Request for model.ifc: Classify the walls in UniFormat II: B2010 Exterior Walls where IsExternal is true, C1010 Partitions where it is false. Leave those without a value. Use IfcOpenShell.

First a look at what the model holds.

```python
import ifcopenshell
import ifcopenshell.util.element

model = ifcopenshell.open("model.ifc")
print(model.schema)
print("classifications:", [c.Name for c in model.by_type("IfcClassification")])
values = [ifcopenshell.util.element.get_pset(e, "Pset_WallCommon", "IsExternal") for e in model.by_type("IfcWall")]
for value in (True, False, None):
    print("IsExternal", value, values.count(value))
```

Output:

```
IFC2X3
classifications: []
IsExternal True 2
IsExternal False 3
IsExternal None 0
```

```python
import ifcopenshell
import ifcopenshell.api.classification
import ifcopenshell.util.element

model = ifcopenshell.open("model.ifc")

# IFC2X3 requires Source and Edition and has no link from the project to the system.
system = model.create_entity("IfcClassification", Source="ASTM", Edition="E1557", Name="UniFormat II")

walls = model.by_type("IfcWall")
external = {e: ifcopenshell.util.element.get_pset(e, "Pset_WallCommon", "IsExternal") for e in walls}
for flag, code, name in ((True, "B2010", "Exterior Walls"), (False, "C1010", "Partitions")):
    products = [e for e in walls if external[e] is flag]
    ifcopenshell.api.classification.add_reference(
        model, products=products, classification=system, identification=code, name=name
    )
    print(code, len(products))

model.write("model_v2.ifc")
```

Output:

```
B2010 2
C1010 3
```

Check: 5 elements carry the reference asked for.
